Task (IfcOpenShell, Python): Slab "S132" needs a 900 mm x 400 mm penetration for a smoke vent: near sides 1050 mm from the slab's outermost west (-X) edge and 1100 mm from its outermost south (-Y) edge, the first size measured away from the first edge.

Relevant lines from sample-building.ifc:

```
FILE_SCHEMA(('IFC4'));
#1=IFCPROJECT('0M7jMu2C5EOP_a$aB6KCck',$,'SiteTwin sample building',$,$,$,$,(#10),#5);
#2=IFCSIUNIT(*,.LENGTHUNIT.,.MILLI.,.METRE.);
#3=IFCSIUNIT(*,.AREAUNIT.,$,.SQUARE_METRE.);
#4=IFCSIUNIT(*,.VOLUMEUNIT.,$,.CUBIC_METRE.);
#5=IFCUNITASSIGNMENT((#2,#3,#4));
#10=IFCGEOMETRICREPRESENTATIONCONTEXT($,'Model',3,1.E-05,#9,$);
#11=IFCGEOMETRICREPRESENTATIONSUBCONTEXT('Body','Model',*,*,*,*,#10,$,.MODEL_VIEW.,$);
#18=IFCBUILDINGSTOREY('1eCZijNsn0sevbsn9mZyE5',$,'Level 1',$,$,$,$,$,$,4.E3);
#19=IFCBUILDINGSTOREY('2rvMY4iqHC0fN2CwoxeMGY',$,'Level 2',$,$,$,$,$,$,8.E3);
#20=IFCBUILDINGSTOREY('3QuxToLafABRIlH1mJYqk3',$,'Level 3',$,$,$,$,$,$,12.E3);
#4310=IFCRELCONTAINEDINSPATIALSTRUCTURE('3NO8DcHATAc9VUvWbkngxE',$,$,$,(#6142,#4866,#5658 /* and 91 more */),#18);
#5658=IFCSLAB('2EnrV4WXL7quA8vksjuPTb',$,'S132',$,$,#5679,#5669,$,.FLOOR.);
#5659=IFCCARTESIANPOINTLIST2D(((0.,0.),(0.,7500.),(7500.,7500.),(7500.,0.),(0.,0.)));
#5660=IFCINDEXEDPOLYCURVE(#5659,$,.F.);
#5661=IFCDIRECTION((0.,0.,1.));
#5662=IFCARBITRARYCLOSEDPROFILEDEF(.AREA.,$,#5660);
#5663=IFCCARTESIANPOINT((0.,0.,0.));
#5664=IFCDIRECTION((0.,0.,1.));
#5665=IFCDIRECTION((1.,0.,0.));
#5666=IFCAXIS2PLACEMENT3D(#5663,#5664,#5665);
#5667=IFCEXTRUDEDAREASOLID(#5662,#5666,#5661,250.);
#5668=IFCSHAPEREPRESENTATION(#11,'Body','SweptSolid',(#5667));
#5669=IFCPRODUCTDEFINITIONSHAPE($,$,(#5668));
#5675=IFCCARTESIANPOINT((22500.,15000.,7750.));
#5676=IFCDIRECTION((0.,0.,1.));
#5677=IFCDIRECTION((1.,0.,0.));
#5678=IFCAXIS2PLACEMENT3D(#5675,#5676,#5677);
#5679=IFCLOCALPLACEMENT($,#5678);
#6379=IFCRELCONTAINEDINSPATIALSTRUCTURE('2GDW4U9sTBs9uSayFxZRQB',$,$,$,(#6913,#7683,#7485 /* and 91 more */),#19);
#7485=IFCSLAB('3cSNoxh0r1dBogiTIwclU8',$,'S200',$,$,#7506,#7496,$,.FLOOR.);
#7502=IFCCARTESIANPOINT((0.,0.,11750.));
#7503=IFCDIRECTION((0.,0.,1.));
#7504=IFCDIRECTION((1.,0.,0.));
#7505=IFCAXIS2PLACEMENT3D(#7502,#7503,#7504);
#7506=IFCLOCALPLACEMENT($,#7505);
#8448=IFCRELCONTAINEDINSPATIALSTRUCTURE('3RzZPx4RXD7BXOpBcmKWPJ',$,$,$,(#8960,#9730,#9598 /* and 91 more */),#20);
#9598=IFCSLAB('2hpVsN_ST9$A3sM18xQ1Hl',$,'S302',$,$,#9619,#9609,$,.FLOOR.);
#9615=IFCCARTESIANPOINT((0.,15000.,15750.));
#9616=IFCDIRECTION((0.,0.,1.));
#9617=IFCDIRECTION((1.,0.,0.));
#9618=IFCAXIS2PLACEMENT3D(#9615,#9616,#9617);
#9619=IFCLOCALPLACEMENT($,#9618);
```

```python
import numpy as np
import ifcopenshell
import ifcopenshell.api.feature
import ifcopenshell.api.geometry
import ifcopenshell.api.root
import ifcopenshell.geom
import ifcopenshell.util.placement
import ifcopenshell.util.representation
import ifcopenshell.util.shape
import ifcopenshell.util.unit

model = ifcopenshell.open("sample-building.ifc")
unit_scale = ifcopenshell.util.unit.calculate_unit_scale(model)
settings = ifcopenshell.geom.settings()


def volume(element):
    """Net volume in cubic metres, openings subtracted."""
    shape = ifcopenshell.geom.create_shape(settings, element)
    return ifcopenshell.util.shape.get_volume(shape.geometry)


slab = model.by_guid("2EnrV4WXL7quA8vksjuPTb")
before = volume(slab)

# Extent in the slab's own axes, in metres. The edges named are its -X and -Y sides.
slab_shape = ifcopenshell.geom.create_shape(settings, slab)
vertices = ifcopenshell.util.shape.get_vertices(slab_shape.geometry)
x_min, y_min, bottom = vertices.min(axis=0)
top = vertices[:, 2].max()

opening = ifcopenshell.api.root.create_entity(model, ifc_class="IfcOpeningElement", name="Smoke vent opening", predefined_type="OPENING")
context = ifcopenshell.util.representation.get_context(model, "Model", "Body", "MODEL_VIEW")
width, depth = 0.9, 0.4
outline = [(0.0, 0.0), (width, 0.0), (width, depth), (0.0, depth), (0.0, 0.0)]
# Overshoot both faces by 50 mm so the cut is clean.
shape = ifcopenshell.api.geometry.add_slab_representation(
    model, context=context, depth=top - bottom + 0.1, polyline=outline
)
ifcopenshell.api.geometry.assign_representation(model, product=opening, representation=shape)

matrix = ifcopenshell.util.placement.get_local_placement(slab.ObjectPlacement)
matrix[:, 3] = matrix @ np.append(np.array([x_min + 1.05, y_min + 1.1, bottom - 0.05]) / unit_scale, 1.0)
ifcopenshell.api.geometry.edit_object_placement(model, product=opening, matrix=matrix, is_si=False)
ifcopenshell.api.feature.add_feature(model, feature=opening, element=slab)

after = volume(slab)

print(f"slab volume {before:.3f} -> {after:.3f} m3")

model.write("sample-building_rev.ifc")
```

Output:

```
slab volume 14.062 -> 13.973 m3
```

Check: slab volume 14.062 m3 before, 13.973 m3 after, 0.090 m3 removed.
